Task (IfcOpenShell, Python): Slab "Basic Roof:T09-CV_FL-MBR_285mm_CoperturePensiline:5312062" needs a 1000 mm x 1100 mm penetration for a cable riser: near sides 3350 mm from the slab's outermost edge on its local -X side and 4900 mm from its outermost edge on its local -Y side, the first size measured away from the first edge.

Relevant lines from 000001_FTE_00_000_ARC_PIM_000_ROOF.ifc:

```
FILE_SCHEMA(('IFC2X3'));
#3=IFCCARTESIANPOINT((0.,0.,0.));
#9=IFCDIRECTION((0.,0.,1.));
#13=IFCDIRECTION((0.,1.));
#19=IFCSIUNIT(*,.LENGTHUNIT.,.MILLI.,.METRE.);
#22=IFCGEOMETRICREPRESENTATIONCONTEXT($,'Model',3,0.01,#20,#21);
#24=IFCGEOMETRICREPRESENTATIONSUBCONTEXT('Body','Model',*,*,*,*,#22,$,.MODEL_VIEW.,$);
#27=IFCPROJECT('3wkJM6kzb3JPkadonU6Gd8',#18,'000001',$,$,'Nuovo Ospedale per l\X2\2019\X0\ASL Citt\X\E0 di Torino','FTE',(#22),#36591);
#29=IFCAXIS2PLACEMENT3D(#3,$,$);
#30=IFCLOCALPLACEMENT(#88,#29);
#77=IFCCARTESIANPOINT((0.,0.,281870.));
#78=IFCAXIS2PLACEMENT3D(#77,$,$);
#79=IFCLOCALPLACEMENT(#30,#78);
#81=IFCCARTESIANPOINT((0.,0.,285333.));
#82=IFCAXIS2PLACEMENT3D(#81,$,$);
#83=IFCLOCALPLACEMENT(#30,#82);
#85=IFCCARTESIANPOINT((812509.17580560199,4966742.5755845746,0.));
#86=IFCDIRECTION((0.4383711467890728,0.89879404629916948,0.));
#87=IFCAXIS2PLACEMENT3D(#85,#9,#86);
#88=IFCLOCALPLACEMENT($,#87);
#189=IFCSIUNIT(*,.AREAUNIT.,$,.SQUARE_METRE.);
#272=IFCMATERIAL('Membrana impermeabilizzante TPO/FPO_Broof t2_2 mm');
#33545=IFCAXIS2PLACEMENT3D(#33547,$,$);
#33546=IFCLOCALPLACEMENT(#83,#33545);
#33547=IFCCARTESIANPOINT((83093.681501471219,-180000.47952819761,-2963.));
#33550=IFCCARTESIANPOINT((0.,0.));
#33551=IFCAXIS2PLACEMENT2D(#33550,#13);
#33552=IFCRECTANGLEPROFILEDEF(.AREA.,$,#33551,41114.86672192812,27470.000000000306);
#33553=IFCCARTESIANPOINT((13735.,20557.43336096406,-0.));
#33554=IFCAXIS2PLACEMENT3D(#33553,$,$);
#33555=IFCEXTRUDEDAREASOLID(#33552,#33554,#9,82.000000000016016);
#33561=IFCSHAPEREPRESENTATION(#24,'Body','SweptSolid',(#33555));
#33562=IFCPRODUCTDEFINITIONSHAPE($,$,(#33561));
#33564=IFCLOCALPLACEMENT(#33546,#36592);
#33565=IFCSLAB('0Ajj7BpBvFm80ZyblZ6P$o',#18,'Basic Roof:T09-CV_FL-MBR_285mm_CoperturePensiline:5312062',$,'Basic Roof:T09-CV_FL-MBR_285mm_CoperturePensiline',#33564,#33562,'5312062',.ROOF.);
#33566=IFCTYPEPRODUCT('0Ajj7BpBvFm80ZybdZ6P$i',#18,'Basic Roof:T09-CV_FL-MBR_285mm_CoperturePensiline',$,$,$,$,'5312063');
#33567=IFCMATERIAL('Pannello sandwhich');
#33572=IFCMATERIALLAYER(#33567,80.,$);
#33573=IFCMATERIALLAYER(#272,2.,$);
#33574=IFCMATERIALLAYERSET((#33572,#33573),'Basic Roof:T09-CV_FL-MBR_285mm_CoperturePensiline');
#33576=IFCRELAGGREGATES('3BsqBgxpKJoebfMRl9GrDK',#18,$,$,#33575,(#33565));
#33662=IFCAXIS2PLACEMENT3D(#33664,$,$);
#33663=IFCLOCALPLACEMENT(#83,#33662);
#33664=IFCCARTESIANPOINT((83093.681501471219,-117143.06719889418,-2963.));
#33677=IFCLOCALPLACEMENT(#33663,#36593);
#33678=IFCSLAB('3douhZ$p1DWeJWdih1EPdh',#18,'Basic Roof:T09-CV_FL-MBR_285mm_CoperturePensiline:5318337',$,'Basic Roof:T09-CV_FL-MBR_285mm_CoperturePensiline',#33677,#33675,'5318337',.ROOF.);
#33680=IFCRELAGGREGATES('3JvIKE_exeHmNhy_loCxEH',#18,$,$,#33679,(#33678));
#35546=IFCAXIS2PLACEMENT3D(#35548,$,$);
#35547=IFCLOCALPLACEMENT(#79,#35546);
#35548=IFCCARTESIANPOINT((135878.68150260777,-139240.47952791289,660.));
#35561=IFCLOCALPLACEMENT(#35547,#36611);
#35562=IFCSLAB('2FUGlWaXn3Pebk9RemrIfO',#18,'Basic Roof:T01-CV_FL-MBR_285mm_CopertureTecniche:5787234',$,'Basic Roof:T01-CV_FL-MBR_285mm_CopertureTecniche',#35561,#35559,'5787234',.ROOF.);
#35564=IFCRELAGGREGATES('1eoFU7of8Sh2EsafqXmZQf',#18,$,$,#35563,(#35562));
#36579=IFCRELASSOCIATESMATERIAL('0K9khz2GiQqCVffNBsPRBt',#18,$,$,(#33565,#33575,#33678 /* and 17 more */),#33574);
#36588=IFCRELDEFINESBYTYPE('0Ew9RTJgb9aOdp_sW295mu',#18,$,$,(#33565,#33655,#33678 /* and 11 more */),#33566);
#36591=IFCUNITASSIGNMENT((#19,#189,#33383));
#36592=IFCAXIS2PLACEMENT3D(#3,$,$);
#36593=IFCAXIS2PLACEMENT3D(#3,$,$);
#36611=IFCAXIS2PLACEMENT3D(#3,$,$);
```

```python
import numpy as np
import ifcopenshell
import ifcopenshell.api.feature
import ifcopenshell.api.geometry
import ifcopenshell.api.root
import ifcopenshell.geom
import ifcopenshell.util.placement
import ifcopenshell.util.representation
import ifcopenshell.util.shape
import ifcopenshell.util.unit

model = ifcopenshell.open("000001_FTE_00_000_ARC_PIM_000_ROOF.ifc")
unit_scale = ifcopenshell.util.unit.calculate_unit_scale(model)
settings = ifcopenshell.geom.settings()


def volume(element):
    """Net volume in cubic metres, openings subtracted."""
    shape = ifcopenshell.geom.create_shape(settings, element)
    return ifcopenshell.util.shape.get_volume(shape.geometry)


slab = model.by_guid("0Ajj7BpBvFm80ZyblZ6P$o")
before = volume(slab)

# Extent in the slab's own axes, in metres. The edges named are its -X and -Y sides.
slab_shape = ifcopenshell.geom.create_shape(settings, slab)
vertices = ifcopenshell.util.shape.get_vertices(slab_shape.geometry)
x_min, y_min, bottom = vertices.min(axis=0)
top = vertices[:, 2].max()

opening = ifcopenshell.api.root.create_entity(model, ifc_class="IfcOpeningElement", name="Cable riser opening")
context = ifcopenshell.util.representation.get_context(model, "Model", "Body", "MODEL_VIEW")
width, depth = 1, 1.1
outline = [(0.0, 0.0), (width, 0.0), (width, depth), (0.0, depth), (0.0, 0.0)]
# Overshoot both faces by 50 mm so the cut is clean.
shape = ifcopenshell.api.geometry.add_slab_representation(
    model, context=context, depth=top - bottom + 0.1, polyline=outline
)
ifcopenshell.api.geometry.assign_representation(model, product=opening, representation=shape)

matrix = ifcopenshell.util.placement.get_local_placement(slab.ObjectPlacement)
matrix[:, 3] = matrix @ np.append(np.array([x_min + 3.35, y_min + 4.9, bottom - 0.05]) / unit_scale, 1.0)
ifcopenshell.api.geometry.edit_object_placement(model, product=opening, matrix=matrix, is_si=False)
ifcopenshell.api.feature.add_feature(model, feature=opening, element=slab)

after = volume(slab)

print(f"slab volume {before:.3f} -> {after:.3f} m3")

model.write("000001_FTE_00_000_ARC_PIM_000_ROOF_v2.ifc")
```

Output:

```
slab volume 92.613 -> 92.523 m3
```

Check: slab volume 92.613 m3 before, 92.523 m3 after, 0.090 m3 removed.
